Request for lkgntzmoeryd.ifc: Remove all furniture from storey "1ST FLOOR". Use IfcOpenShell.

First a look at what the model holds.

```python
import ifcopenshell
import ifcopenshell.util.element

model = ifcopenshell.open("lkgntzmoeryd.ifc")
print(model.schema)
storey = next(s for s in model.by_type("IfcBuildingStorey") if s.Name == "1ST FLOOR")
furniture = [e for e in ifcopenshell.util.element.get_decomposition(storey) if e.is_a("IfcFurnishingElement")]
seen = {}
for e in furniture:
    element_type = ifcopenshell.util.element.get_type(e)
    name = element_type.Name if element_type not in (None, e) else None
    seen[name] = seen.get(name, 0) + 1
for name, count in sorted(seen.items(), key=str):
    print(count, "x", name)
```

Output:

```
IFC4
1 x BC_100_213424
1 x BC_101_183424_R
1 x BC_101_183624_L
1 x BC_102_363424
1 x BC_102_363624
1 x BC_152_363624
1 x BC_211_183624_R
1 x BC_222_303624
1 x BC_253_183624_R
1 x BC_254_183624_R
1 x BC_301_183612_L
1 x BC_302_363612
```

```python
import ifcopenshell
import ifcopenshell.api.root
import ifcopenshell.util.element

model = ifcopenshell.open("lkgntzmoeryd.ifc")

storey = next(s for s in model.by_type("IfcBuildingStorey") if s.Name == "1ST FLOOR")
furniture = [e for e in ifcopenshell.util.element.get_decomposition(storey) if e.is_a("IfcFurnishingElement")]

for e in furniture:
    ifcopenshell.api.root.remove_product(model, product=e)
print(len(furniture), "removed")

model.write("lkgntzmoeryd_v2.ifc")
```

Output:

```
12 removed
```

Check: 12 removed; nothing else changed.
